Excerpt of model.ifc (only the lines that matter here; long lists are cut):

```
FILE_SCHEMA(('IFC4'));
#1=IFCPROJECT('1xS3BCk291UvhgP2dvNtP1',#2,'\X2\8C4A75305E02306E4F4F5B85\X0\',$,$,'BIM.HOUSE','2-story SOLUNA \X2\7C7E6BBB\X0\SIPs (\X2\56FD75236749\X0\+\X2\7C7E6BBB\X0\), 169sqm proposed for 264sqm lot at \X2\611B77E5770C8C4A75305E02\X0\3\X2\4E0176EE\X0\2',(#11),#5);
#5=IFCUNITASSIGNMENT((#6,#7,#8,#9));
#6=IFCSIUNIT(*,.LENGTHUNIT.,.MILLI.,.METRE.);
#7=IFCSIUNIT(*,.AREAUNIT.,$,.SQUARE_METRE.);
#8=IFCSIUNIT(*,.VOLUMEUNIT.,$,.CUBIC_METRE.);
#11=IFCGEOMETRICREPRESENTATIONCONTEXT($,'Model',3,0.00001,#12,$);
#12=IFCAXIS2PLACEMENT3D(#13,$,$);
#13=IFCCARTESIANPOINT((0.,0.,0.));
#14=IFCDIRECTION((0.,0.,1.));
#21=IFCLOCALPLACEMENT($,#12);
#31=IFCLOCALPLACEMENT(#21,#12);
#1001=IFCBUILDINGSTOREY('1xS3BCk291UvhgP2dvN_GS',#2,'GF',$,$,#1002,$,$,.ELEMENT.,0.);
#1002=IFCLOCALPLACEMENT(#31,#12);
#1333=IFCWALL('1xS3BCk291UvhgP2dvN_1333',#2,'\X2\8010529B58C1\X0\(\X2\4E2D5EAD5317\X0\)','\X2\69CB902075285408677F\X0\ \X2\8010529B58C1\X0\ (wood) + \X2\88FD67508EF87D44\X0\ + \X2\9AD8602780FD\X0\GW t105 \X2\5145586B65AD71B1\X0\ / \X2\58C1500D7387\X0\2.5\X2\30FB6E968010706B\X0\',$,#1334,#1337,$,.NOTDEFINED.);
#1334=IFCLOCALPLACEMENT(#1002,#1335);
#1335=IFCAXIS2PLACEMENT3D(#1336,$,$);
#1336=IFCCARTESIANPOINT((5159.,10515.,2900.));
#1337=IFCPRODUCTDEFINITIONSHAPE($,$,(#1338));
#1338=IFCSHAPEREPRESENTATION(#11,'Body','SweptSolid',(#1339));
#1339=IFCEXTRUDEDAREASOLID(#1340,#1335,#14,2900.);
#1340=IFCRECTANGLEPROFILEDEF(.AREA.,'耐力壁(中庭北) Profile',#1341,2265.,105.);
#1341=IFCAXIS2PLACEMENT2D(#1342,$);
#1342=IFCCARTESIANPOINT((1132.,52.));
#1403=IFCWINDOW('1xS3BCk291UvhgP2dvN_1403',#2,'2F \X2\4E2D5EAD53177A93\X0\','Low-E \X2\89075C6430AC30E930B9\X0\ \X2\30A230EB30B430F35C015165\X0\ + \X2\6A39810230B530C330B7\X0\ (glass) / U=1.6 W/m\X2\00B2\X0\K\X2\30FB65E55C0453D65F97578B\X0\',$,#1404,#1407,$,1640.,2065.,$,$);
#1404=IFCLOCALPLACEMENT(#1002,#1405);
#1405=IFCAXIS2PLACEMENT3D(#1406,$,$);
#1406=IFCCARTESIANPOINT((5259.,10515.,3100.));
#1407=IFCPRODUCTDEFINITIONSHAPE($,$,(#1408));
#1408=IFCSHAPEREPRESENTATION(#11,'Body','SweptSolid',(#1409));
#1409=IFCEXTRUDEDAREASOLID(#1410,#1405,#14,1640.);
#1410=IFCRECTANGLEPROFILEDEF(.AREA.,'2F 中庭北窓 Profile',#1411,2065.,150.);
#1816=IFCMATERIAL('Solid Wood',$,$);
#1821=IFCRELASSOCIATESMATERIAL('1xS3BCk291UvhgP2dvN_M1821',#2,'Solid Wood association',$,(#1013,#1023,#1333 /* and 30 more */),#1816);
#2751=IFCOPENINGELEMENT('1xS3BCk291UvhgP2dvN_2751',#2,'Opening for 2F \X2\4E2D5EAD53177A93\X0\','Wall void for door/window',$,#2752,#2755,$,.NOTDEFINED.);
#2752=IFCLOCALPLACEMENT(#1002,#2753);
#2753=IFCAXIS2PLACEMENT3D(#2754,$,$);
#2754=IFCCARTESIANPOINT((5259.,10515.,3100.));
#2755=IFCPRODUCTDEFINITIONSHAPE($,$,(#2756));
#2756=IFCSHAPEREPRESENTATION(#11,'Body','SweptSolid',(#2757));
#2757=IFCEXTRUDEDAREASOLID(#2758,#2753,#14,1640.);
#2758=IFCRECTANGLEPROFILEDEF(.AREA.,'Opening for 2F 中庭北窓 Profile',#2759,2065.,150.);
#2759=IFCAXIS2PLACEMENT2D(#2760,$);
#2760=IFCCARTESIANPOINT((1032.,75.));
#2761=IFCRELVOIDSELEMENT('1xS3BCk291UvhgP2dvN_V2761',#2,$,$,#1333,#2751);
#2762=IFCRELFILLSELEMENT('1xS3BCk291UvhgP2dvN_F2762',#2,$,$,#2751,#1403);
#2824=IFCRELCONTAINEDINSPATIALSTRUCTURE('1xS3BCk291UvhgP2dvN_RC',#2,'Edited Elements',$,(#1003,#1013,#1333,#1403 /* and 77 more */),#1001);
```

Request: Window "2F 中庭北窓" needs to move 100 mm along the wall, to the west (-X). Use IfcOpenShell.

```python
import ifcopenshell
import ifcopenshell.api.geometry
import ifcopenshell.util.placement

model = ifcopenshell.open("model.ifc")

window = model.by_guid("1xS3BCk291UvhgP2dvN_1403")
opening = window.FillsVoids[0].RelatingOpeningElement
wall = opening.VoidsElements[0].RelatingBuildingElement

wall_matrix = ifcopenshell.util.placement.get_local_placement(wall.ObjectPlacement)
shift = wall_matrix[:3, 0] * -100.0
before = ifcopenshell.util.placement.get_local_placement(window.ObjectPlacement)[:3, 3].copy()

# The window is not placed relative to its opening, so move both.
for product in (opening, window):
    matrix = ifcopenshell.util.placement.get_local_placement(product.ObjectPlacement)
    matrix[:3, 3] += shift
    ifcopenshell.api.geometry.edit_object_placement(model, product=product, matrix=matrix, is_si=False)

after = ifcopenshell.util.placement.get_local_placement(window.ObjectPlacement)[:3, 3]
print("window moved by", (after - before).round(3) + 0.0)

model.write("model_v2.ifc")
```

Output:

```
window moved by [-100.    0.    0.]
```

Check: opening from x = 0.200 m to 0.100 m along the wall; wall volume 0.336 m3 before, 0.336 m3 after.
